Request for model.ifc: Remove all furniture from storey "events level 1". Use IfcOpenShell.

First a look at what the model holds.

```python
import ifcopenshell
import ifcopenshell.util.element

model = ifcopenshell.open("model.ifc")
print(model.schema)
storey = next(s for s in model.by_type("IfcBuildingStorey") if s.Name == "events level 1")
furniture = [e for e in ifcopenshell.util.element.get_decomposition(storey) if e.is_a("IfcFurnishingElement")]
seen = {}
for e in furniture:
    element_type = ifcopenshell.util.element.get_type(e)
    name = element_type.Name if element_type not in (None, e) else None
    seen[name] = seen.get(name, 0) + 1
for name, count in sorted(seen.items(), key=str):
    print(count, "x", name)
```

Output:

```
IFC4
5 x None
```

```python
import ifcopenshell
import ifcopenshell.api.root
import ifcopenshell.util.element

model = ifcopenshell.open("model.ifc")

storey = next(s for s in model.by_type("IfcBuildingStorey") if s.Name == "events level 1")
furniture = [e for e in ifcopenshell.util.element.get_decomposition(storey) if e.is_a("IfcFurnishingElement")]

for e in furniture:
    ifcopenshell.api.root.remove_product(model, product=e)
print(len(furniture), "removed")

model.write("model-out.ifc")
```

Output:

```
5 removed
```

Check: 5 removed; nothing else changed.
